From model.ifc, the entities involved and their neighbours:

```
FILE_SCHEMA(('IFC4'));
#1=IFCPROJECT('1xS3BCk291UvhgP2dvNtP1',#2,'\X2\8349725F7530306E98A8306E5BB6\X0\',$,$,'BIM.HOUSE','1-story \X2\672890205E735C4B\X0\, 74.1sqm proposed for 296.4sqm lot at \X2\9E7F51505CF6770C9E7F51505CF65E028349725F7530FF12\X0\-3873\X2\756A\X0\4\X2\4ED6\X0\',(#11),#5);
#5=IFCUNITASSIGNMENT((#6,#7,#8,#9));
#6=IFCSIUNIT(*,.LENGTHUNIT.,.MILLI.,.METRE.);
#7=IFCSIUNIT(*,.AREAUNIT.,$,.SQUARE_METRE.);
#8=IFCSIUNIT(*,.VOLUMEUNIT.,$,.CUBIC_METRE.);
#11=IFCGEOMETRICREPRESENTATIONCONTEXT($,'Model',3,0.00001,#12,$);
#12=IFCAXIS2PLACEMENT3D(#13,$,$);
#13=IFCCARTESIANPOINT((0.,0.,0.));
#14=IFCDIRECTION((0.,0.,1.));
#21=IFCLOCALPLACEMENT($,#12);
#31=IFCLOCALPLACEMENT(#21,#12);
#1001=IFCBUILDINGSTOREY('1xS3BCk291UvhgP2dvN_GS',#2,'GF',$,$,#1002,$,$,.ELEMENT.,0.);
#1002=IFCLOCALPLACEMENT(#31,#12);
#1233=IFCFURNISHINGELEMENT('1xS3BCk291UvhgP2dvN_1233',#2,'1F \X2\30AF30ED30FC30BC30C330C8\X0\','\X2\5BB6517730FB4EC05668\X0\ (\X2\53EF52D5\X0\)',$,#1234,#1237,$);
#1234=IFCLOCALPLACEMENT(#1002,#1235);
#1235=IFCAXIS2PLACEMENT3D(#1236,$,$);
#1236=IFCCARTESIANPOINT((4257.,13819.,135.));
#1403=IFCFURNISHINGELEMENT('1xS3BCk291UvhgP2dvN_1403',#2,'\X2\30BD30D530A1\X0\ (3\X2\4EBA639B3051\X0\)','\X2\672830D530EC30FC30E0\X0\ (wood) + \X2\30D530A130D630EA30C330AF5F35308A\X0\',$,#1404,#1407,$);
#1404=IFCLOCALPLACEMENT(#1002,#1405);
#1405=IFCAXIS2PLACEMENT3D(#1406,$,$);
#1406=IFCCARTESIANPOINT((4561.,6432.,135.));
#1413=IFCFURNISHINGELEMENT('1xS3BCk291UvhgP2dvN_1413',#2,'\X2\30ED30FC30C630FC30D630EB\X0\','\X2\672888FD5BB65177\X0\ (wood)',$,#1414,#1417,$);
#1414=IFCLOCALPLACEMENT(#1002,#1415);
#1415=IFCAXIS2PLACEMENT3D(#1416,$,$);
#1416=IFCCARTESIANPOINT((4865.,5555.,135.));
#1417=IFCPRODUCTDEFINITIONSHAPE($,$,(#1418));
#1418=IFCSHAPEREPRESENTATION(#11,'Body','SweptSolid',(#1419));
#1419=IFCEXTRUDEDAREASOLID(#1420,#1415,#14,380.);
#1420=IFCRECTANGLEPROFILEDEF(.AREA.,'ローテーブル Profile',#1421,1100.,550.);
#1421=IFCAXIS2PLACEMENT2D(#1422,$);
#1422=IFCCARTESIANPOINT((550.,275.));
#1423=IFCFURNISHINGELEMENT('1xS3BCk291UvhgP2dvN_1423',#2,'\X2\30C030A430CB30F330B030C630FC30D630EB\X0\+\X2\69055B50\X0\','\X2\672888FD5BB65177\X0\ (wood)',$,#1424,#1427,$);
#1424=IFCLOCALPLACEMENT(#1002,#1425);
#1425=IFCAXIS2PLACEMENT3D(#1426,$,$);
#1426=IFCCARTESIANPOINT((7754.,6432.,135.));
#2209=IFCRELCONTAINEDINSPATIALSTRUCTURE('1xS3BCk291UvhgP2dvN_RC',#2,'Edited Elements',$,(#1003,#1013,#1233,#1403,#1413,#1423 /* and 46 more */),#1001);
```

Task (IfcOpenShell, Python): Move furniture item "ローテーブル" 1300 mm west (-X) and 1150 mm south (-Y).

```python
import ifcopenshell
import ifcopenshell.api.geometry
import ifcopenshell.util.placement
import ifcopenshell.util.unit

model = ifcopenshell.open("model.ifc")
unit_scale = ifcopenshell.util.unit.calculate_unit_scale(model)

item = model.by_guid("1xS3BCk291UvhgP2dvN_1413")
matrix = ifcopenshell.util.placement.get_local_placement(item.ObjectPlacement)
matrix[0, 3] -= 1.3 / unit_scale
matrix[1, 3] -= 1.15 / unit_scale
ifcopenshell.api.geometry.edit_object_placement(model, product=item, matrix=matrix, is_si=False)

print(ifcopenshell.util.placement.get_local_placement(item.ObjectPlacement).round(3) + 0.0)

model.write("model_edited.ifc")
```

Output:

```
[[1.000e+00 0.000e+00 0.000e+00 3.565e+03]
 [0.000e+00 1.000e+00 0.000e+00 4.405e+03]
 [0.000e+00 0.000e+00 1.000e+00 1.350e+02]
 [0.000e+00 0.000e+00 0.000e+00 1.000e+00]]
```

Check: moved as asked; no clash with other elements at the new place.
